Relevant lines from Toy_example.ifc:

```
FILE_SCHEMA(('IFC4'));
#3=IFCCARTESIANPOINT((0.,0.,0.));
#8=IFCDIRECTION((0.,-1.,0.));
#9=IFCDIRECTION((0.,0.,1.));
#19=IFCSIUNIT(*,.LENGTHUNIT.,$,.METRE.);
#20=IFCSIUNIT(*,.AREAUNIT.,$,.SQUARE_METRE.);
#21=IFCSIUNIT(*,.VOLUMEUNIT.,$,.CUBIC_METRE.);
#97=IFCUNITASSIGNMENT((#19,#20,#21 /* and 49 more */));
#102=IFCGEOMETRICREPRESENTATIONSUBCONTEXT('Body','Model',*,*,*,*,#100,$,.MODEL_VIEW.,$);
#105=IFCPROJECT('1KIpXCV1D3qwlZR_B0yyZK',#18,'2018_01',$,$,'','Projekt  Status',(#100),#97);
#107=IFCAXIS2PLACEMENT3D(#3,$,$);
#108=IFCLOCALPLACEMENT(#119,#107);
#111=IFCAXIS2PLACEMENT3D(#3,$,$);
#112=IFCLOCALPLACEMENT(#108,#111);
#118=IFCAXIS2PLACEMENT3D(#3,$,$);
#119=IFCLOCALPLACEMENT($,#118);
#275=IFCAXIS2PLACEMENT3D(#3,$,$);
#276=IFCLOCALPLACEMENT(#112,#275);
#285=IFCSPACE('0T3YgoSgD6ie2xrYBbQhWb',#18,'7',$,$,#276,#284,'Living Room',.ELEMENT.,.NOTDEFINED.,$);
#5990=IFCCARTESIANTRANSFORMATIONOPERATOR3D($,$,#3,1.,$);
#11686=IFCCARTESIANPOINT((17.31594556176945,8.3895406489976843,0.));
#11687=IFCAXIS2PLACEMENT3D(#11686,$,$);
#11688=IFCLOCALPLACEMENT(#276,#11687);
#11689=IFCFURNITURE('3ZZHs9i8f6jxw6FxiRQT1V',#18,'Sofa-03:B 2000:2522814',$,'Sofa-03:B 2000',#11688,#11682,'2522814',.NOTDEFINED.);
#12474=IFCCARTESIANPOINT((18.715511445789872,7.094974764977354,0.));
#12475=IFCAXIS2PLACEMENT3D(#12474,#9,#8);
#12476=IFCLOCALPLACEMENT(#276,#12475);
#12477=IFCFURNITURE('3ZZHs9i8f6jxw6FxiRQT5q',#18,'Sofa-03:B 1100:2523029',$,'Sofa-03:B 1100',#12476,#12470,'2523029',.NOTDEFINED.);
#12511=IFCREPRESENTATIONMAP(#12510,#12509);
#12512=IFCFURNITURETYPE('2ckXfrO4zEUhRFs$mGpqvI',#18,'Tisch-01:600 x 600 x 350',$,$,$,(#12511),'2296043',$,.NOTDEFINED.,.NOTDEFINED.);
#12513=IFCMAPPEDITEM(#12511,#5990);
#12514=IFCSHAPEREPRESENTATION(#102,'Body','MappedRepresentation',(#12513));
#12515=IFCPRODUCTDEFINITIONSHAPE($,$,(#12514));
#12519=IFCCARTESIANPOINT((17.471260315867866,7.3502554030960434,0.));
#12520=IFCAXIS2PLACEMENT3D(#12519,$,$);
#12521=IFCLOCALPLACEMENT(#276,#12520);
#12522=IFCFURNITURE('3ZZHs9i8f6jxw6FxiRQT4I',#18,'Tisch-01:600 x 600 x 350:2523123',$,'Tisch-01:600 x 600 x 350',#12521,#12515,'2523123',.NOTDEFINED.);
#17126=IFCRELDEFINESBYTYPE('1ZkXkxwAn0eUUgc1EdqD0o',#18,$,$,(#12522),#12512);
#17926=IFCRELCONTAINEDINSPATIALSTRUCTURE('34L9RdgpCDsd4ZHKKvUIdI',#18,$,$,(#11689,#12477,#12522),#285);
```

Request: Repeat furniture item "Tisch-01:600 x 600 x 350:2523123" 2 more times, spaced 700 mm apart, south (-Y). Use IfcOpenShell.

```python
import numpy as np
import ifcopenshell
import ifcopenshell.api.geometry
import ifcopenshell.api.root
import ifcopenshell.util.element
import ifcopenshell.util.placement

model = ifcopenshell.open("Toy_example.ifc")


def reuse_history(source, copy):
    """copy_class also copies each property set's owner history, people and application; keep the originals."""
    for rel in copy.IsDefinedBy:
        if rel.is_a("IfcRelDefinesByProperties") and (history := rel.RelatingPropertyDefinition.OwnerHistory):
            rel.RelatingPropertyDefinition.OwnerHistory = source.OwnerHistory
            ifcopenshell.util.element.remove_deep2(model, history)


source = model.by_guid("3ZZHs9i8f6jxw6FxiRQT4I")
base = ifcopenshell.util.placement.get_local_placement(source.ObjectPlacement)
step = np.array([0.0, -1.0, 0.0]) * 0.7

for i in range(1, 3):
    copy = ifcopenshell.api.root.copy_class(model, product=source)
    copy.Representation = ifcopenshell.util.element.copy_deep(
        model, source.Representation, exclude=["IfcGeometricRepresentationContext", "IfcRepresentationMap"]
    )
    copy.Name = "Tisch-01:600 x 600 x 350"
    copy.Tag = None
    reuse_history(source, copy)
    matrix = base.copy()
    matrix[:3, 3] += i * step
    print("added at", matrix[:3, 3].round(3) + 0.0)
    ifcopenshell.api.geometry.edit_object_placement(model, product=copy, matrix=matrix, is_si=False)

model.write("Toy_example_updated.ifc")
```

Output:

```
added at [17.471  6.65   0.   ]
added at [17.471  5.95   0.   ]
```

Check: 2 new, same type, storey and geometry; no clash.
